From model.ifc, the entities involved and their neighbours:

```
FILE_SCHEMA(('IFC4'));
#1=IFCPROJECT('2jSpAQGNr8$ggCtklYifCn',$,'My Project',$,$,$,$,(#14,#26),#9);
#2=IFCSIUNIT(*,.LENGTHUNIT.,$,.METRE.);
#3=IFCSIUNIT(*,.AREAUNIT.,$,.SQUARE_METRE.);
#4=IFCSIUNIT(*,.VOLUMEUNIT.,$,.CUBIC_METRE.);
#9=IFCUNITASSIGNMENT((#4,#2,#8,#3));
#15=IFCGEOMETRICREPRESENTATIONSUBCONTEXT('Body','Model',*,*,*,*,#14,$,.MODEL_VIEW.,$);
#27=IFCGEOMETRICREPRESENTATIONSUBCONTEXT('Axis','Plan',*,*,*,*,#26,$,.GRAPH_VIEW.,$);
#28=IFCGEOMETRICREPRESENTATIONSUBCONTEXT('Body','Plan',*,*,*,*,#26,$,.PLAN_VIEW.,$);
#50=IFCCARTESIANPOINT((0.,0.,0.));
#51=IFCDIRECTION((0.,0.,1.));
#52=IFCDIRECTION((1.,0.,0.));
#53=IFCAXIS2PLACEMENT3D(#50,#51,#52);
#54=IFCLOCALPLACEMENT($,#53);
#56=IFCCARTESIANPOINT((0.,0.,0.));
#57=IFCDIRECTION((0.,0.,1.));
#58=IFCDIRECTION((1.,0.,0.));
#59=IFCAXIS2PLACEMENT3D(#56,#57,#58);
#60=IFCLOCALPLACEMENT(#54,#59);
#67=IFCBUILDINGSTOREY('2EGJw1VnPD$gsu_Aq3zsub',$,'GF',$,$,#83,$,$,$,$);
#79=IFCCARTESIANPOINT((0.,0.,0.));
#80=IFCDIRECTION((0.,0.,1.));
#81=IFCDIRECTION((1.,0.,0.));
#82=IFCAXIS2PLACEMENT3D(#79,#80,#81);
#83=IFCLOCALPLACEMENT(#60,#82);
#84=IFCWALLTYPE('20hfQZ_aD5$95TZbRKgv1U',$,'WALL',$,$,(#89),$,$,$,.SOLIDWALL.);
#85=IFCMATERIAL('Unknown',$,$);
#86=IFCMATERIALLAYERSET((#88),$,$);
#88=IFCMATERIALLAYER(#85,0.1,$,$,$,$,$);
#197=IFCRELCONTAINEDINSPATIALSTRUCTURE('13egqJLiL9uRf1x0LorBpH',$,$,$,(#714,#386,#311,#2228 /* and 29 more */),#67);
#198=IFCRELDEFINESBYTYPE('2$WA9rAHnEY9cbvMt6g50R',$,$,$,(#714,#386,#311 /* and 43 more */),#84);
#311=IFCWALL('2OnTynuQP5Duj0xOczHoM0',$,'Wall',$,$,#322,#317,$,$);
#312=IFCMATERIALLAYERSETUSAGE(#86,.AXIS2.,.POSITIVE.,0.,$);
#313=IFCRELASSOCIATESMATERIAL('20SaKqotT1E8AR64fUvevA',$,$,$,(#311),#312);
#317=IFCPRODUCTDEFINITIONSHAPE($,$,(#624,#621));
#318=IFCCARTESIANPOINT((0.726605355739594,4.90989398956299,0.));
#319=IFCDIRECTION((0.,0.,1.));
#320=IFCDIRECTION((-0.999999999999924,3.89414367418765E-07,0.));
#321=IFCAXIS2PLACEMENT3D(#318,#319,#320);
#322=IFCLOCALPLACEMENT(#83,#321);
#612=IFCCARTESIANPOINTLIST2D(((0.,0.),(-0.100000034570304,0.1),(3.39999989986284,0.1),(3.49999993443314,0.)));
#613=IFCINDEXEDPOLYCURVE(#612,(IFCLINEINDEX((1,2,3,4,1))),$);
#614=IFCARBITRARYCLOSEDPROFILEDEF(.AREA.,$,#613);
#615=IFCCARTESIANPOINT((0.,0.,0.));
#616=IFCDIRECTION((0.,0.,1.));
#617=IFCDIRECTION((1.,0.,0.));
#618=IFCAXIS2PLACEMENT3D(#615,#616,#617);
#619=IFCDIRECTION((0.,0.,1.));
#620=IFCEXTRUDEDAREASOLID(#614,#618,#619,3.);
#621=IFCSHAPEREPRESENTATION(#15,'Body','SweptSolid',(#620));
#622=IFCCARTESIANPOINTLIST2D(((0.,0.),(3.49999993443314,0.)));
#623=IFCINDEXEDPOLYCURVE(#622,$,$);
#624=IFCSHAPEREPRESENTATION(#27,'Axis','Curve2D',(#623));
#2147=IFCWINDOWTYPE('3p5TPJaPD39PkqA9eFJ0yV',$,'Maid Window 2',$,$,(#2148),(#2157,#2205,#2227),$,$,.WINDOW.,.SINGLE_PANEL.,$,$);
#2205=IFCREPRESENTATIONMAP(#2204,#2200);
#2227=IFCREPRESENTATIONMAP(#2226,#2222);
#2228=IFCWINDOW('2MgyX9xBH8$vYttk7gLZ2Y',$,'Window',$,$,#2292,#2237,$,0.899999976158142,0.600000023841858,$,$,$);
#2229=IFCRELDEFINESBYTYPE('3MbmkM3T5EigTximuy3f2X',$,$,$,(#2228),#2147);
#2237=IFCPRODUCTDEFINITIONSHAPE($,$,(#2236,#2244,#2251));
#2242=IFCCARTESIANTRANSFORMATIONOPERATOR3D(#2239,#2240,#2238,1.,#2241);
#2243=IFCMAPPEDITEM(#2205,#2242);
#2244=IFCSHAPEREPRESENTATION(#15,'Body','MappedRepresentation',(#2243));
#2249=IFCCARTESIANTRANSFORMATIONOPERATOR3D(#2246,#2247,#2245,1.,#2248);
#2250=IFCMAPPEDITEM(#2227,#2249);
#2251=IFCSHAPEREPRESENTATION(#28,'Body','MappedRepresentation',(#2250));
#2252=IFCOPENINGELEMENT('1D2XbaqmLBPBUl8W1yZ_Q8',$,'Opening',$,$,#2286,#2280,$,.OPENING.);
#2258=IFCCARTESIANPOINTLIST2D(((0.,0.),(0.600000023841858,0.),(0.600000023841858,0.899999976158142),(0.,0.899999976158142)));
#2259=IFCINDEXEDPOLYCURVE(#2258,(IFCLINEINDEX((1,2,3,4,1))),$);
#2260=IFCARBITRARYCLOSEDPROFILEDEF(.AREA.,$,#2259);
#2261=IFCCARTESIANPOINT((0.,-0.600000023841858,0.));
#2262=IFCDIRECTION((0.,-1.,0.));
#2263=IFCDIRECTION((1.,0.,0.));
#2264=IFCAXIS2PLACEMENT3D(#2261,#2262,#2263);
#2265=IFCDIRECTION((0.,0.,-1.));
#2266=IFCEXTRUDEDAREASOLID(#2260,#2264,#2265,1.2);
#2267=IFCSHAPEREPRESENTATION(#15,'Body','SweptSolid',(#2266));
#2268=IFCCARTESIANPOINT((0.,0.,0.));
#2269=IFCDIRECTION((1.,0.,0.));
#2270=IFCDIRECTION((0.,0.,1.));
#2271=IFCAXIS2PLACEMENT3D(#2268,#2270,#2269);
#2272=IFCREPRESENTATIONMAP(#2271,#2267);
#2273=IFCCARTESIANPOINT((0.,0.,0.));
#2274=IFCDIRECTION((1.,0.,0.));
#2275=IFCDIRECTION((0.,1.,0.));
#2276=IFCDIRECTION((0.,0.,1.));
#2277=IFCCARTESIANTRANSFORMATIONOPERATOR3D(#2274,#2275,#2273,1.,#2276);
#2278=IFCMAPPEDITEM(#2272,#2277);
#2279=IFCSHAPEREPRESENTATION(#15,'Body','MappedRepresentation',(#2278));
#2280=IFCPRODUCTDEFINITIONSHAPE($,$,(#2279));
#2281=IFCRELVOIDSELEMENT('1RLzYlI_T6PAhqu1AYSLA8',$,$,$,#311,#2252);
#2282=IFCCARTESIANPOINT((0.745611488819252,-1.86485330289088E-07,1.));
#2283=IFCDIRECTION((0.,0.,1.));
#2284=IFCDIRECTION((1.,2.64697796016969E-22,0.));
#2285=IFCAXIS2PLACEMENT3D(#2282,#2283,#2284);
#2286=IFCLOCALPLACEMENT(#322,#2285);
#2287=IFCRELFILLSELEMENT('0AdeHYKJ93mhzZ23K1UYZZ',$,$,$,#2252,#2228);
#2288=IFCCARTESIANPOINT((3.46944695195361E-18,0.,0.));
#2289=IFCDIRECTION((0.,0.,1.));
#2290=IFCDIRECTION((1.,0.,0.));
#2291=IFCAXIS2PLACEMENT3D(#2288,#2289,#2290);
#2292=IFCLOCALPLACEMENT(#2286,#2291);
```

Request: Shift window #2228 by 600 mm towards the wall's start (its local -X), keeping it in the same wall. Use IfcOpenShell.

```python
import ifcopenshell
import ifcopenshell.api.geometry
import ifcopenshell.util.placement

model = ifcopenshell.open("model.ifc")

window = model.by_guid("2MgyX9xBH8$vYttk7gLZ2Y")
opening = window.FillsVoids[0].RelatingOpeningElement
wall = opening.VoidsElements[0].RelatingBuildingElement

wall_matrix = ifcopenshell.util.placement.get_local_placement(wall.ObjectPlacement)
shift = wall_matrix[:3, 0] * -0.6
before = ifcopenshell.util.placement.get_local_placement(window.ObjectPlacement)[:3, 3].copy()

# The window is placed relative to its opening, so it follows when the opening moves.
matrix = ifcopenshell.util.placement.get_local_placement(opening.ObjectPlacement)
matrix[:3, 3] += shift
ifcopenshell.api.geometry.edit_object_placement(
    model, product=opening, matrix=matrix, is_si=False, should_transform_children=True
)

after = ifcopenshell.util.placement.get_local_placement(window.ObjectPlacement)[:3, 3]
print("window moved by", (after - before).round(3) + 0.0)

model.write("model_rev.ifc")
```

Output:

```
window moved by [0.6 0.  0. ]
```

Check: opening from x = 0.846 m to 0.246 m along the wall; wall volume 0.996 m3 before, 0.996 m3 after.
